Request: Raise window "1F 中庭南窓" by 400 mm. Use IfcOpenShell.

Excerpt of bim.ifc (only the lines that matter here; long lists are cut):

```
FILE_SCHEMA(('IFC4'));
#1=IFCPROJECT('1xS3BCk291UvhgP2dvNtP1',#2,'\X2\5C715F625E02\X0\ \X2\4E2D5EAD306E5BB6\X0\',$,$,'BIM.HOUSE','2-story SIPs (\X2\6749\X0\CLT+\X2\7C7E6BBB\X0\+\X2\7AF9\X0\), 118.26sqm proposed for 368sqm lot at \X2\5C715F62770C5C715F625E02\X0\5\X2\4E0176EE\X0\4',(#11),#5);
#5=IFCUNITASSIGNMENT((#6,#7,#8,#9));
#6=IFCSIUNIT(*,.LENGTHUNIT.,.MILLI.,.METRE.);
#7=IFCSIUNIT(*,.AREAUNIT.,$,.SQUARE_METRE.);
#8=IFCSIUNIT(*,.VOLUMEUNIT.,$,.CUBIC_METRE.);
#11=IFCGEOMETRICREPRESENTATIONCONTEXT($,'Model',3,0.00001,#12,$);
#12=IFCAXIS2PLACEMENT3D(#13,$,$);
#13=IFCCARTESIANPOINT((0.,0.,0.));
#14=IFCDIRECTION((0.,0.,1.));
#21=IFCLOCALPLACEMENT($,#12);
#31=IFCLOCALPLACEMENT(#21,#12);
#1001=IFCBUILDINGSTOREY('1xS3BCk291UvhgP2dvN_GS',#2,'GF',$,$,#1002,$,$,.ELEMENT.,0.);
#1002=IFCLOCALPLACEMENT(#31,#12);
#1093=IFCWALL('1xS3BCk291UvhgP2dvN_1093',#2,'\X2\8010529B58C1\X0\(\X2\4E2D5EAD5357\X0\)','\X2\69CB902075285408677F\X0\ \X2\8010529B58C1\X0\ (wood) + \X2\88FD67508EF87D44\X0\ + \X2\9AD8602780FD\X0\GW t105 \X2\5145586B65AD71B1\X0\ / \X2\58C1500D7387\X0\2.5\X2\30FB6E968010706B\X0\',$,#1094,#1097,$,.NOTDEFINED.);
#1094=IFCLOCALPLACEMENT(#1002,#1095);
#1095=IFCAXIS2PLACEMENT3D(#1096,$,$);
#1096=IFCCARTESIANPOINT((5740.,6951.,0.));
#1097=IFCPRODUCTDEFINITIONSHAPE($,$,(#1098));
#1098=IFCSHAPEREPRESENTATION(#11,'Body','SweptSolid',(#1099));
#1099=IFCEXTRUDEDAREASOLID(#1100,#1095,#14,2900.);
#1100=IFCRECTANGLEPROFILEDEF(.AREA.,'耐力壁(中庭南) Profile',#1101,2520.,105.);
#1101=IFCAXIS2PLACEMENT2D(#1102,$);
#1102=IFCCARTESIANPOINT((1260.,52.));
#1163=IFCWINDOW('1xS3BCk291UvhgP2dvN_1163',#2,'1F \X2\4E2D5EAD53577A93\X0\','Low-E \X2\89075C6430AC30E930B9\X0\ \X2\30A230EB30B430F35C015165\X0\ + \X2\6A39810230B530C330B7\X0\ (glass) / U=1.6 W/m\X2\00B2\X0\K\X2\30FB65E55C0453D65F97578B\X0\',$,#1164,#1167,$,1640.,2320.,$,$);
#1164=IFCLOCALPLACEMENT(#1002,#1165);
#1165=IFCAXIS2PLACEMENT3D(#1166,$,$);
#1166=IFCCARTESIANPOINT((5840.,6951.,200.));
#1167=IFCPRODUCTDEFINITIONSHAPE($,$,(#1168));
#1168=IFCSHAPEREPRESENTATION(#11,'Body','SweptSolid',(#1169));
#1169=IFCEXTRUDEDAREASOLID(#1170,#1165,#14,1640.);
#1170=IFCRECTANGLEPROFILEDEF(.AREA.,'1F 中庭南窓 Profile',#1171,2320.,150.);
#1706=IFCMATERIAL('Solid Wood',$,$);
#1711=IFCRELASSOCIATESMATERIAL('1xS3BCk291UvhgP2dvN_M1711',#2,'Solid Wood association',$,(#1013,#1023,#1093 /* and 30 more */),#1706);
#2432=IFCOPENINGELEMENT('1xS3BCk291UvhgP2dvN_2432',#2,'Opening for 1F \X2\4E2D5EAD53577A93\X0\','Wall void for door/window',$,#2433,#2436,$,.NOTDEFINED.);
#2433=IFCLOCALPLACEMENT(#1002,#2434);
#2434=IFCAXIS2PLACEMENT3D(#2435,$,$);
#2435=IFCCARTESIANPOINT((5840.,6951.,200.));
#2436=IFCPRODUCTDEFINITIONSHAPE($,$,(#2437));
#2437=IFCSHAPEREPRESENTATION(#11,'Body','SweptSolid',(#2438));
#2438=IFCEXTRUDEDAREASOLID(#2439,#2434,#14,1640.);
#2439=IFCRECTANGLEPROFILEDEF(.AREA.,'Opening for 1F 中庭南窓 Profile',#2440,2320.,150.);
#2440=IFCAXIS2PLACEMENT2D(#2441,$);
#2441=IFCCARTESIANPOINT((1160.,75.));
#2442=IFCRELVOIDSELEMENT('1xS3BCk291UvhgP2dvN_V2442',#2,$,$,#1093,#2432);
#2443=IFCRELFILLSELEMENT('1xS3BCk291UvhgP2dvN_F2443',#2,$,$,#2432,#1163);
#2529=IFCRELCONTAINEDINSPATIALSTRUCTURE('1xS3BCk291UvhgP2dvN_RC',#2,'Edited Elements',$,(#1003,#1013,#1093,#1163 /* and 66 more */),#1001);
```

```python
import numpy as np
import ifcopenshell
import ifcopenshell.api.geometry
import ifcopenshell.util.placement
import ifcopenshell.util.unit

model = ifcopenshell.open("bim.ifc")
unit_scale = ifcopenshell.util.unit.calculate_unit_scale(model)

window = model.by_guid("1xS3BCk291UvhgP2dvN_1163")
opening = window.FillsVoids[0].RelatingOpeningElement
dz = 0.4 / unit_scale

shift = np.array([0.0, 0.0, dz])
# The window is not placed relative to its opening, so move both.
for product in (opening, window):
    matrix = ifcopenshell.util.placement.get_local_placement(product.ObjectPlacement)
    matrix[:3, 3] += shift
    ifcopenshell.api.geometry.edit_object_placement(model, product=product, matrix=matrix, is_si=False)

print(f"moved by {dz * unit_scale:+.3f} m")

model.write("bim_updated.ifc")
```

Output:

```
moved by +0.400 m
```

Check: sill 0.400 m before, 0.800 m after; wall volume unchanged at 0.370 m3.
